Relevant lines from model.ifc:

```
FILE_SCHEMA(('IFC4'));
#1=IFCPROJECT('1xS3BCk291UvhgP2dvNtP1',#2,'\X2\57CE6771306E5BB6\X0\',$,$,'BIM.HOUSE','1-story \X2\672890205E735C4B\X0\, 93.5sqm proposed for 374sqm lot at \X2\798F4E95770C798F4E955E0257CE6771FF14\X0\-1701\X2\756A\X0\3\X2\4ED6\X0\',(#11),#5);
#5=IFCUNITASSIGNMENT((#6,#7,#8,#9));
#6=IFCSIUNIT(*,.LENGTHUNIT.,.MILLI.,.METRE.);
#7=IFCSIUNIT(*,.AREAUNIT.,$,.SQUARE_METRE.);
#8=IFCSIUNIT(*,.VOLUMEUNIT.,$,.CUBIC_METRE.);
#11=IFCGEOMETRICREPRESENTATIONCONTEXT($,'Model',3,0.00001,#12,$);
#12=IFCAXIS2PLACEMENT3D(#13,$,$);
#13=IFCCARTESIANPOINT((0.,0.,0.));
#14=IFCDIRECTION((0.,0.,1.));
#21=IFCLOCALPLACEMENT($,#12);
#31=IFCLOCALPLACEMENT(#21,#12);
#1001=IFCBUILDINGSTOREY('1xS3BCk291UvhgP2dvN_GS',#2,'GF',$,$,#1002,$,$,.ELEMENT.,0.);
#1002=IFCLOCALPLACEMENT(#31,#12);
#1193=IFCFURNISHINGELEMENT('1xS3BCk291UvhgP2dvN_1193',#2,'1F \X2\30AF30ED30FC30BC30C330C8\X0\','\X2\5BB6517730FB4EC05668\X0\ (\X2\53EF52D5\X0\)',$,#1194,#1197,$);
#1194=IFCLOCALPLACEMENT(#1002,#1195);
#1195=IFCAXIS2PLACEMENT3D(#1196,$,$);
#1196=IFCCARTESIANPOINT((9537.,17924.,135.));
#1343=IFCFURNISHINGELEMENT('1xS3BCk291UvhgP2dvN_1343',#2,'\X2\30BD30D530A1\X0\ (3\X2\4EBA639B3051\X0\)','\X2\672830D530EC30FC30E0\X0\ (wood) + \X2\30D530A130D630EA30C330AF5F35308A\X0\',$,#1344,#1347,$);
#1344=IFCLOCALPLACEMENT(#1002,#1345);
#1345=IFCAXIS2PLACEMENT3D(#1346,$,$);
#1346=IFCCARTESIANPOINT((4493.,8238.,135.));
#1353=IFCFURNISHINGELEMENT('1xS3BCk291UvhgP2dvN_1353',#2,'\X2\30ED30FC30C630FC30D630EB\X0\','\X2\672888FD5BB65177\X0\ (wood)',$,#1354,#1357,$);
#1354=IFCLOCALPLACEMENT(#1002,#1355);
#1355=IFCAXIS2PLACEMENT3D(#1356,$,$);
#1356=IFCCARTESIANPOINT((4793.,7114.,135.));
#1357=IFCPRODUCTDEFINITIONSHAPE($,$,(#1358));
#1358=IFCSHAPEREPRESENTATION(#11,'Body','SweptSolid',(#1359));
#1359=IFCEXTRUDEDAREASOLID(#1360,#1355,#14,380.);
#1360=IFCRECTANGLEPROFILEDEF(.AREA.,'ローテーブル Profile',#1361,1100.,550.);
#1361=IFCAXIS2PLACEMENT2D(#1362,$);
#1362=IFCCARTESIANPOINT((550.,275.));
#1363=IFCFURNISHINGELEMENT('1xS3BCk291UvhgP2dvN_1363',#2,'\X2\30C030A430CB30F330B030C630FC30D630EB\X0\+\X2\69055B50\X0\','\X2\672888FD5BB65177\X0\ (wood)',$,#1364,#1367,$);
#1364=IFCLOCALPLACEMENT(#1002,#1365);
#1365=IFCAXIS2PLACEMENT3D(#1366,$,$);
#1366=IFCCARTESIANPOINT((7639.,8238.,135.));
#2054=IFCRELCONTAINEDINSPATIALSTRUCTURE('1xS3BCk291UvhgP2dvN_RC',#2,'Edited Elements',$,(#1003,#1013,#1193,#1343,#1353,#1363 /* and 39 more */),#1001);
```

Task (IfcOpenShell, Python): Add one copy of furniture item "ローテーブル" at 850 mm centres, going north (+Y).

```python
import numpy as np
import ifcopenshell
import ifcopenshell.api.geometry
import ifcopenshell.api.root
import ifcopenshell.util.element
import ifcopenshell.util.placement

model = ifcopenshell.open("model.ifc")


def reuse_history(source, copy):
    """copy_class also copies each property set's owner history, people and application; keep the originals."""
    for rel in copy.IsDefinedBy:
        if rel.is_a("IfcRelDefinesByProperties") and (history := rel.RelatingPropertyDefinition.OwnerHistory):
            rel.RelatingPropertyDefinition.OwnerHistory = source.OwnerHistory
            ifcopenshell.util.element.remove_deep2(model, history)


source = model.by_guid("1xS3BCk291UvhgP2dvN_1353")
base = ifcopenshell.util.placement.get_local_placement(source.ObjectPlacement)
step = np.array([0.0, 1.0, 0.0]) * 850.0

for i in range(1, 2):
    copy = ifcopenshell.api.root.copy_class(model, product=source)
    copy.Representation = ifcopenshell.util.element.copy_deep(
        model, source.Representation, exclude=["IfcGeometricRepresentationContext", "IfcRepresentationMap"]
    )
    reuse_history(source, copy)
    matrix = base.copy()
    matrix[:3, 3] += i * step
    print("added at", matrix[:3, 3].round(3) + 0.0)
    ifcopenshell.api.geometry.edit_object_placement(model, product=copy, matrix=matrix, is_si=False)

model.write("model_edited.ifc")
```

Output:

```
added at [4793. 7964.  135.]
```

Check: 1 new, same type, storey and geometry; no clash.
